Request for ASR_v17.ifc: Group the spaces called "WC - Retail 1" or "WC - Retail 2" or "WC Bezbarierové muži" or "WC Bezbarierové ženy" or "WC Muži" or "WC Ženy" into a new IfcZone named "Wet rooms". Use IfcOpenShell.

First a look at what the model holds.

```python
import ifcopenshell

model = ifcopenshell.open("ASR_v17.ifc")
print(model.schema)
seen = {}
for space in model.by_type("IfcSpace"):
    seen[space.LongName] = seen.get(space.LongName, 0) + 1
for name, count in sorted(seen.items(), key=str):
    print(count, "x", name)
print("zones:", [z.Name for z in model.by_type("IfcZone")][:20])
```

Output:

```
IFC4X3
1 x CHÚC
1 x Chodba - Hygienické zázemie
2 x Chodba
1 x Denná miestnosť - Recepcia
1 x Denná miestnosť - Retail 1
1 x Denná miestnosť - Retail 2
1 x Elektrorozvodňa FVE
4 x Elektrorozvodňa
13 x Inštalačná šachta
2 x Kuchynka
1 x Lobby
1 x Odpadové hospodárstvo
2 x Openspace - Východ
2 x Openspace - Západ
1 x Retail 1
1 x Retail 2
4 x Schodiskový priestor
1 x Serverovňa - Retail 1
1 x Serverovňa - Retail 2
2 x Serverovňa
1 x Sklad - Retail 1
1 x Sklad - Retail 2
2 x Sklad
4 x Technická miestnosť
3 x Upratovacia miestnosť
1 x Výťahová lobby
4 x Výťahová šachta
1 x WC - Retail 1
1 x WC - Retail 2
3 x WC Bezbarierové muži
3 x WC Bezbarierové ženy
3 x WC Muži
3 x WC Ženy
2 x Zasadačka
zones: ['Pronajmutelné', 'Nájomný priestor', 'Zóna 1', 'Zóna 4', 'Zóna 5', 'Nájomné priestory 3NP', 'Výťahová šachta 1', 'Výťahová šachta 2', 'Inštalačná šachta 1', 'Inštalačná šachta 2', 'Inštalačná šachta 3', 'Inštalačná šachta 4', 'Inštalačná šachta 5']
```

```python
import ifcopenshell
import ifcopenshell.api.group
import ifcopenshell.api.root

model = ifcopenshell.open("ASR_v17.ifc")

names = {"WC - Retail 1", "WC - Retail 2", "WC Bezbarierové muži", "WC Bezbarierové ženy", "WC Muži", "WC Ženy"}
spaces = [s for s in model.by_type("IfcSpace") if s.LongName in names]

zone = ifcopenshell.api.root.create_entity(model, ifc_class="IfcZone", name="Wet rooms")
ifcopenshell.api.group.assign_group(model, products=spaces, group=zone)
print(len(spaces), "spaces in", zone.Name)

model.write("ASR_v17_v2.ifc")
```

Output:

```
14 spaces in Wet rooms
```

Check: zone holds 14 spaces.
